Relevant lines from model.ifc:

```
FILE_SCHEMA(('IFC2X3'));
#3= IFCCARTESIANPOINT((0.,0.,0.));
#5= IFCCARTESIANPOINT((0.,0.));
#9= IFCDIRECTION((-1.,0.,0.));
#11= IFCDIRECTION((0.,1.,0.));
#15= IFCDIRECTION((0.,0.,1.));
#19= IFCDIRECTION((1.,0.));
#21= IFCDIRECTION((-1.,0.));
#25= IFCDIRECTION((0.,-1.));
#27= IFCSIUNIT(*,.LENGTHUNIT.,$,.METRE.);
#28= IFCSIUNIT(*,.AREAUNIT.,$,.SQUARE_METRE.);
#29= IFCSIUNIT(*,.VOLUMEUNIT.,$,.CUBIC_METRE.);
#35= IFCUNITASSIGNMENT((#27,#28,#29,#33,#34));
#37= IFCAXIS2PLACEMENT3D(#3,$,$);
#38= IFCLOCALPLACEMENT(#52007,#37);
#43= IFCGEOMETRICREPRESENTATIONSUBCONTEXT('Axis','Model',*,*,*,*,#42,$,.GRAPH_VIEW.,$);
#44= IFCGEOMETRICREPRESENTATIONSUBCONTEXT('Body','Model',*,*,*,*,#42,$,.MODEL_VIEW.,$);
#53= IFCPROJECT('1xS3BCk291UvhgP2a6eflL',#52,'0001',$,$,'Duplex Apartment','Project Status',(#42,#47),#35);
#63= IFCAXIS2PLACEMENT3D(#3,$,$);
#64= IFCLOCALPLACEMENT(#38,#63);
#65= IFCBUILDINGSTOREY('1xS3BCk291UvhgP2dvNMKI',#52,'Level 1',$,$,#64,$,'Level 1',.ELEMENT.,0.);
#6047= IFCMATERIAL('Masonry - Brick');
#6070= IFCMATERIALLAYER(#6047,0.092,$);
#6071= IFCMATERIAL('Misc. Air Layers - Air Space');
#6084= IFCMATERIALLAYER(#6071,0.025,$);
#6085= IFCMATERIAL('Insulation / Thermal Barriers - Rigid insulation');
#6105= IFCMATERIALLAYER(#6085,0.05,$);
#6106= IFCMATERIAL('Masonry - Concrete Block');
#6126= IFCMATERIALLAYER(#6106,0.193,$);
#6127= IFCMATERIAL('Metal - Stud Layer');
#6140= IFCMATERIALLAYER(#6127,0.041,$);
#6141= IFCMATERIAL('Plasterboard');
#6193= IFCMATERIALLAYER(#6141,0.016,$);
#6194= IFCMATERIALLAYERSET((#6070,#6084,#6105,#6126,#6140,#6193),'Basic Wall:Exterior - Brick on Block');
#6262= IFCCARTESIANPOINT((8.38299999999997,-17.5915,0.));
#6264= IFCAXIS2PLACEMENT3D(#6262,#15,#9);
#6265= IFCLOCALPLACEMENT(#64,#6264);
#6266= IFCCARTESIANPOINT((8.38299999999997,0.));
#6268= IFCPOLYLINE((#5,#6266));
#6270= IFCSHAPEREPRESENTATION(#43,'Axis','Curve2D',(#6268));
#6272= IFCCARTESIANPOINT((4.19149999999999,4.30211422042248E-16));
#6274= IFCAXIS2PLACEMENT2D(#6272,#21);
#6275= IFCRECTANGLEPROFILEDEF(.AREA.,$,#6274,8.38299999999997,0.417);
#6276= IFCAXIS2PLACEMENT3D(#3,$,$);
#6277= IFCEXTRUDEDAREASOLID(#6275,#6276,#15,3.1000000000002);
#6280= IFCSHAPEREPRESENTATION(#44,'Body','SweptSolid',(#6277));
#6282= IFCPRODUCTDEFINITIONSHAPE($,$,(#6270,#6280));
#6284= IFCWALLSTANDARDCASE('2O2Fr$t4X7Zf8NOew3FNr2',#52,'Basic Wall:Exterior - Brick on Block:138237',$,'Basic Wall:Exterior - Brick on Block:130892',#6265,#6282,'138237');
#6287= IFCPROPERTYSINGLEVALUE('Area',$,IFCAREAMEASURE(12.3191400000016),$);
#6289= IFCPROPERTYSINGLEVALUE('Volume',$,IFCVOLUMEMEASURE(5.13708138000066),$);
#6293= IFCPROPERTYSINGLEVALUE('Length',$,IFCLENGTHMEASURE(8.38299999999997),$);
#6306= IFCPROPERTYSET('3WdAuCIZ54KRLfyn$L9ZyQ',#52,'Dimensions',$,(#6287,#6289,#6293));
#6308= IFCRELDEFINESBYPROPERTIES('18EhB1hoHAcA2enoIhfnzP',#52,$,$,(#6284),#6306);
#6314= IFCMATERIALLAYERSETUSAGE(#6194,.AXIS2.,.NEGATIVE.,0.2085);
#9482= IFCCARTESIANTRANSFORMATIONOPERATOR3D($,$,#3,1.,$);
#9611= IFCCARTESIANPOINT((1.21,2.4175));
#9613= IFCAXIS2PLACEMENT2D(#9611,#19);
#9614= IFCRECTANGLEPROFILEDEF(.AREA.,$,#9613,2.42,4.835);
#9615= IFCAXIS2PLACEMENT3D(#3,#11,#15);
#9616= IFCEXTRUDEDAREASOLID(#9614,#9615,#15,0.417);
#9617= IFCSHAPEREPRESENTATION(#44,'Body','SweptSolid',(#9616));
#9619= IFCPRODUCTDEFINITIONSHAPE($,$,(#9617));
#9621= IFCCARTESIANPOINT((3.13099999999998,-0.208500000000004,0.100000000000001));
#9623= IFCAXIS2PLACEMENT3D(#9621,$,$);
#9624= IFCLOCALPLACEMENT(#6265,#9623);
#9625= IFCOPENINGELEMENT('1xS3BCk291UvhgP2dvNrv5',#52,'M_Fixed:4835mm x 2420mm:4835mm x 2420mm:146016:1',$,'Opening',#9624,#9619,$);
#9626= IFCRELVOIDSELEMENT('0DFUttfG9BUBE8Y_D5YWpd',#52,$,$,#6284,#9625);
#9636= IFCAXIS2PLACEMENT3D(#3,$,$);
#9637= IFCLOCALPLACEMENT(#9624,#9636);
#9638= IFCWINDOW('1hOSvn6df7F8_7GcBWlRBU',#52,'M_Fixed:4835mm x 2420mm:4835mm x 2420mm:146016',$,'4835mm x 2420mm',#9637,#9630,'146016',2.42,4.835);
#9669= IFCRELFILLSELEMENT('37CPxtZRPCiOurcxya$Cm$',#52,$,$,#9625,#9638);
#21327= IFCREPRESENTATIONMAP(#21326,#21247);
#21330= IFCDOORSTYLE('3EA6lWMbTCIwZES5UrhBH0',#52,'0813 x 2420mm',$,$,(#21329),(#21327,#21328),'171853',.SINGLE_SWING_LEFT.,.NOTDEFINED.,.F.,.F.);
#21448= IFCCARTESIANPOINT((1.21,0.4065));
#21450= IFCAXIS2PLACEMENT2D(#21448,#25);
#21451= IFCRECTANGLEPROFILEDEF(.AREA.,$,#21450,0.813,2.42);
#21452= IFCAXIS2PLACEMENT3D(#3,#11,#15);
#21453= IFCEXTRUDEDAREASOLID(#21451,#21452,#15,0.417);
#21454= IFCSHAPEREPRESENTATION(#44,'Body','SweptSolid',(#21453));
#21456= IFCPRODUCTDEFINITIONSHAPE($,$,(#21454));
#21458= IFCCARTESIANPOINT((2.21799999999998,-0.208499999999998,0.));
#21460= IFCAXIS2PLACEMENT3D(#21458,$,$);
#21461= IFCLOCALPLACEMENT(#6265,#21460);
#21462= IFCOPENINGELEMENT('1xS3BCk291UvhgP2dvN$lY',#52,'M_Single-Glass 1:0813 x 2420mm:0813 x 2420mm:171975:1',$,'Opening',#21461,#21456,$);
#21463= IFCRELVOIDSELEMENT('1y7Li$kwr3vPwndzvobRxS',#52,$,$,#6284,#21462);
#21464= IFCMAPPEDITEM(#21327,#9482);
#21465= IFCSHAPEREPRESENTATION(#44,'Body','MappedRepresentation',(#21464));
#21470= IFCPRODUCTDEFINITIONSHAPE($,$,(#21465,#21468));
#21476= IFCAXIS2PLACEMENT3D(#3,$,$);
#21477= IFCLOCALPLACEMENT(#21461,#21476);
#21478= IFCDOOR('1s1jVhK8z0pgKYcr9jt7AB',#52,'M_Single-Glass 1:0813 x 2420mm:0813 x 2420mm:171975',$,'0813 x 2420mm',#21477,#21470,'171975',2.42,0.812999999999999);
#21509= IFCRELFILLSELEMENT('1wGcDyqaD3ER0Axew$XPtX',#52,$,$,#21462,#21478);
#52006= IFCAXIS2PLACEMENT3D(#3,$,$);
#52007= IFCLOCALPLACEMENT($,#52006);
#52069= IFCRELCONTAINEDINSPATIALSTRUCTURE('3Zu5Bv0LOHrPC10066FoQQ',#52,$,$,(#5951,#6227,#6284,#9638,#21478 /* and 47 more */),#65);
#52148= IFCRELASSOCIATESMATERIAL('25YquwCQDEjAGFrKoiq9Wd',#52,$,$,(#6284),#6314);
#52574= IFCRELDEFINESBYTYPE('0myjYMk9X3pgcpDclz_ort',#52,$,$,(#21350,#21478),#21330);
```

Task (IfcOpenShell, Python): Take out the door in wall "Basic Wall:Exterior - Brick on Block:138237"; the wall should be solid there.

```python
import ifcopenshell
import ifcopenshell.api.feature
import ifcopenshell.api.pset
import ifcopenshell.api.root
import ifcopenshell.geom
import ifcopenshell.util.element
import ifcopenshell.util.shape
import ifcopenshell.util.unit

model = ifcopenshell.open("model.ifc")
area_scale = ifcopenshell.util.unit.calculate_unit_scale(model, "AREAUNIT")
volume_scale = ifcopenshell.util.unit.calculate_unit_scale(model, "VOLUMEUNIT")
settings = ifcopenshell.geom.settings()


def volume(element):
    """Net volume in cubic metres, openings subtracted."""
    shape = ifcopenshell.geom.create_shape(settings, element)
    return ifcopenshell.util.shape.get_volume(shape.geometry)


door = model.by_guid("1s1jVhK8z0pgKYcr9jt7AB")
opening = door.FillsVoids[0].RelatingOpeningElement
wall = opening.VoidsElements[0].RelatingBuildingElement
before = volume(wall)

ifcopenshell.api.root.remove_product(model, product=door)
ifcopenshell.api.feature.remove_feature(model, feature=opening)

after = volume(wall)
thickness = 0.417  # wall thickness in metres

# Update the wall's stored quantities.
pset = model.by_id(ifcopenshell.util.element.get_pset(wall, "Dimensions", should_inherit=False)["id"])
ifcopenshell.api.pset.edit_pset(model, pset=pset, properties={
    "Area": model.create_entity("IfcAreaMeasure", after / thickness / area_scale),
    "Volume": model.create_entity("IfcVolumeMeasure", after / volume_scale),
})

print(f"wall volume {before:.3f} -> {after:.3f} m3")

model.write("model_v2.ifc")
```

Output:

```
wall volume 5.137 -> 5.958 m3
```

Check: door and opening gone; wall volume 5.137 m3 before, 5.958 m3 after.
